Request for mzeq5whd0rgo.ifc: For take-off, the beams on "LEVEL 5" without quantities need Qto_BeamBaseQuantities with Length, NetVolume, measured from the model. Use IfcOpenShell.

First a look at what the model holds.

```python
import ifcopenshell
import ifcopenshell.util.element
import ifcopenshell.util.unit

model = ifcopenshell.open("mzeq5whd0rgo.ifc")
print(model.schema)
for unit_type in ("LENGTHUNIT", "AREAUNIT", "VOLUMEUNIT"):
    print(unit_type, ifcopenshell.util.unit.calculate_unit_scale(model, unit_type))
storey = next(s for s in model.by_type("IfcBuildingStorey") if s.Name == "LEVEL 5")
beams = [e for e in ifcopenshell.util.element.get_decomposition(storey) if e.is_a("IfcBeam")]
for e in sorted(beams, key=lambda e: e.id()):
    print(e.id(), e.is_a(), e.Name, list(ifcopenshell.util.element.get_psets(e, qtos_only=True)), sep=" | ")
```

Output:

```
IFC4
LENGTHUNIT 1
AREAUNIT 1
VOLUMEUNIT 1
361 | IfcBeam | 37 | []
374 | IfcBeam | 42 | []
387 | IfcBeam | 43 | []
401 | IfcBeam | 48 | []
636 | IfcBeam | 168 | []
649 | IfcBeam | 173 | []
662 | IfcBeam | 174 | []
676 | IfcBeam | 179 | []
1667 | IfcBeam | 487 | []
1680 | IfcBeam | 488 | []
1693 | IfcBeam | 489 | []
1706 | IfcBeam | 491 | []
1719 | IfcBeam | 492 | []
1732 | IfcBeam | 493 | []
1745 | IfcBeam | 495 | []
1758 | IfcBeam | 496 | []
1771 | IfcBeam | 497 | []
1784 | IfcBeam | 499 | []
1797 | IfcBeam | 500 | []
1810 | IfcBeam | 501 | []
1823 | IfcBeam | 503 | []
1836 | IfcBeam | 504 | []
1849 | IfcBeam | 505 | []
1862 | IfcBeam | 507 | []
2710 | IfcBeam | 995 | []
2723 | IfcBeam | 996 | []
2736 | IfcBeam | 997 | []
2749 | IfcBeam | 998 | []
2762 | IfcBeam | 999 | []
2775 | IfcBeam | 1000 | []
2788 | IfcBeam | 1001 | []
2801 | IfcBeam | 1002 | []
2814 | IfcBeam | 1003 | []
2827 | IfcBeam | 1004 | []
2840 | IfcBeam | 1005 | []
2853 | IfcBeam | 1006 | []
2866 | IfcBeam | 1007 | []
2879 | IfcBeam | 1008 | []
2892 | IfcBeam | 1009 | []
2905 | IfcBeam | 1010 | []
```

```python
import ifcopenshell
import ifcopenshell.api.pset
import ifcopenshell.geom
import ifcopenshell.util.element
import ifcopenshell.util.shape
import ifcopenshell.util.unit

model = ifcopenshell.open("mzeq5whd0rgo.ifc")
unit_scale = ifcopenshell.util.unit.calculate_unit_scale(model)
volume_scale = ifcopenshell.util.unit.calculate_unit_scale(model, "VOLUMEUNIT")
settings = ifcopenshell.geom.settings()

storey = next(s for s in model.by_type("IfcBuildingStorey") if s.Name == "LEVEL 5")
beams = [e for e in ifcopenshell.util.element.get_decomposition(storey) if e.is_a("IfcBeam")]

for e in sorted(beams, key=lambda e: e.id()):
    if ifcopenshell.util.element.get_psets(e, qtos_only=True, should_inherit=False):
        continue
    # Geometry comes back in metres, in the element's own axes.
    shape = ifcopenshell.geom.create_shape(settings, e)
    values = {
        "Length": ifcopenshell.util.shape.get_max_xyz(shape.geometry) / unit_scale,
        "NetVolume": ifcopenshell.util.shape.get_volume(shape.geometry) / volume_scale,
    }
    qto = ifcopenshell.api.pset.add_qto(model, product=e, name="Qto_BeamBaseQuantities")
    ifcopenshell.api.pset.edit_qto(model, qto=qto, properties=values)
    print(e.id(), {k: round(v, 3) for k, v in values.items()})

model.write("mzeq5whd0rgo_updated.ifc")
```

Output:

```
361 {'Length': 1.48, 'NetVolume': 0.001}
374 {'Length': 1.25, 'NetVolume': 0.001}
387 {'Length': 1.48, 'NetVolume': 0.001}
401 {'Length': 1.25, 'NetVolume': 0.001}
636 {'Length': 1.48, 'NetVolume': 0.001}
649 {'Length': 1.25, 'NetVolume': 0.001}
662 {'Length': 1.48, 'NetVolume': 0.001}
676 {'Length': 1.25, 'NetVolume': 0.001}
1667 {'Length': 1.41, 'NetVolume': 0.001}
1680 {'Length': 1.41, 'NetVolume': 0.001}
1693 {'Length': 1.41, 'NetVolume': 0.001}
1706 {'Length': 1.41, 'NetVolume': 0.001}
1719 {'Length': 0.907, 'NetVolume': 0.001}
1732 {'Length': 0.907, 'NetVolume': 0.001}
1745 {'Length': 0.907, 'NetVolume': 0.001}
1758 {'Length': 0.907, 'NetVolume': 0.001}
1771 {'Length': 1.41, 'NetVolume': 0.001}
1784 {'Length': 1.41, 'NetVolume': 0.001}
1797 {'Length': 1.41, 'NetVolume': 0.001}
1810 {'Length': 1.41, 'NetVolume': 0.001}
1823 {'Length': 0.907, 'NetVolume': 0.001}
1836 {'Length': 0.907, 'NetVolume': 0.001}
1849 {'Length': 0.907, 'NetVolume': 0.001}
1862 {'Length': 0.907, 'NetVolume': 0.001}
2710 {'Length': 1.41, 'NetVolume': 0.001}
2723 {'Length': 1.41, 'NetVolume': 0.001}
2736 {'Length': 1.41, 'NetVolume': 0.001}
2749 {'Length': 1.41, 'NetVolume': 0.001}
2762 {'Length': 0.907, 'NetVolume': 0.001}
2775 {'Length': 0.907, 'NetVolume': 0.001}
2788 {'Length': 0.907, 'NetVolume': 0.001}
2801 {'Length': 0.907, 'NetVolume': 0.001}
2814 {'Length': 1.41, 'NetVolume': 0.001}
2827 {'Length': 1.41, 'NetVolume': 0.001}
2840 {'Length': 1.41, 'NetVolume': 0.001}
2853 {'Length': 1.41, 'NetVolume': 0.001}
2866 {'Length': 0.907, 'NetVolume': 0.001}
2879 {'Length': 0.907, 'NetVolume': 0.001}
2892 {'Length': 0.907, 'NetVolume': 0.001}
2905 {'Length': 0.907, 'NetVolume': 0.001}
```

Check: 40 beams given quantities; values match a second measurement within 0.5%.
